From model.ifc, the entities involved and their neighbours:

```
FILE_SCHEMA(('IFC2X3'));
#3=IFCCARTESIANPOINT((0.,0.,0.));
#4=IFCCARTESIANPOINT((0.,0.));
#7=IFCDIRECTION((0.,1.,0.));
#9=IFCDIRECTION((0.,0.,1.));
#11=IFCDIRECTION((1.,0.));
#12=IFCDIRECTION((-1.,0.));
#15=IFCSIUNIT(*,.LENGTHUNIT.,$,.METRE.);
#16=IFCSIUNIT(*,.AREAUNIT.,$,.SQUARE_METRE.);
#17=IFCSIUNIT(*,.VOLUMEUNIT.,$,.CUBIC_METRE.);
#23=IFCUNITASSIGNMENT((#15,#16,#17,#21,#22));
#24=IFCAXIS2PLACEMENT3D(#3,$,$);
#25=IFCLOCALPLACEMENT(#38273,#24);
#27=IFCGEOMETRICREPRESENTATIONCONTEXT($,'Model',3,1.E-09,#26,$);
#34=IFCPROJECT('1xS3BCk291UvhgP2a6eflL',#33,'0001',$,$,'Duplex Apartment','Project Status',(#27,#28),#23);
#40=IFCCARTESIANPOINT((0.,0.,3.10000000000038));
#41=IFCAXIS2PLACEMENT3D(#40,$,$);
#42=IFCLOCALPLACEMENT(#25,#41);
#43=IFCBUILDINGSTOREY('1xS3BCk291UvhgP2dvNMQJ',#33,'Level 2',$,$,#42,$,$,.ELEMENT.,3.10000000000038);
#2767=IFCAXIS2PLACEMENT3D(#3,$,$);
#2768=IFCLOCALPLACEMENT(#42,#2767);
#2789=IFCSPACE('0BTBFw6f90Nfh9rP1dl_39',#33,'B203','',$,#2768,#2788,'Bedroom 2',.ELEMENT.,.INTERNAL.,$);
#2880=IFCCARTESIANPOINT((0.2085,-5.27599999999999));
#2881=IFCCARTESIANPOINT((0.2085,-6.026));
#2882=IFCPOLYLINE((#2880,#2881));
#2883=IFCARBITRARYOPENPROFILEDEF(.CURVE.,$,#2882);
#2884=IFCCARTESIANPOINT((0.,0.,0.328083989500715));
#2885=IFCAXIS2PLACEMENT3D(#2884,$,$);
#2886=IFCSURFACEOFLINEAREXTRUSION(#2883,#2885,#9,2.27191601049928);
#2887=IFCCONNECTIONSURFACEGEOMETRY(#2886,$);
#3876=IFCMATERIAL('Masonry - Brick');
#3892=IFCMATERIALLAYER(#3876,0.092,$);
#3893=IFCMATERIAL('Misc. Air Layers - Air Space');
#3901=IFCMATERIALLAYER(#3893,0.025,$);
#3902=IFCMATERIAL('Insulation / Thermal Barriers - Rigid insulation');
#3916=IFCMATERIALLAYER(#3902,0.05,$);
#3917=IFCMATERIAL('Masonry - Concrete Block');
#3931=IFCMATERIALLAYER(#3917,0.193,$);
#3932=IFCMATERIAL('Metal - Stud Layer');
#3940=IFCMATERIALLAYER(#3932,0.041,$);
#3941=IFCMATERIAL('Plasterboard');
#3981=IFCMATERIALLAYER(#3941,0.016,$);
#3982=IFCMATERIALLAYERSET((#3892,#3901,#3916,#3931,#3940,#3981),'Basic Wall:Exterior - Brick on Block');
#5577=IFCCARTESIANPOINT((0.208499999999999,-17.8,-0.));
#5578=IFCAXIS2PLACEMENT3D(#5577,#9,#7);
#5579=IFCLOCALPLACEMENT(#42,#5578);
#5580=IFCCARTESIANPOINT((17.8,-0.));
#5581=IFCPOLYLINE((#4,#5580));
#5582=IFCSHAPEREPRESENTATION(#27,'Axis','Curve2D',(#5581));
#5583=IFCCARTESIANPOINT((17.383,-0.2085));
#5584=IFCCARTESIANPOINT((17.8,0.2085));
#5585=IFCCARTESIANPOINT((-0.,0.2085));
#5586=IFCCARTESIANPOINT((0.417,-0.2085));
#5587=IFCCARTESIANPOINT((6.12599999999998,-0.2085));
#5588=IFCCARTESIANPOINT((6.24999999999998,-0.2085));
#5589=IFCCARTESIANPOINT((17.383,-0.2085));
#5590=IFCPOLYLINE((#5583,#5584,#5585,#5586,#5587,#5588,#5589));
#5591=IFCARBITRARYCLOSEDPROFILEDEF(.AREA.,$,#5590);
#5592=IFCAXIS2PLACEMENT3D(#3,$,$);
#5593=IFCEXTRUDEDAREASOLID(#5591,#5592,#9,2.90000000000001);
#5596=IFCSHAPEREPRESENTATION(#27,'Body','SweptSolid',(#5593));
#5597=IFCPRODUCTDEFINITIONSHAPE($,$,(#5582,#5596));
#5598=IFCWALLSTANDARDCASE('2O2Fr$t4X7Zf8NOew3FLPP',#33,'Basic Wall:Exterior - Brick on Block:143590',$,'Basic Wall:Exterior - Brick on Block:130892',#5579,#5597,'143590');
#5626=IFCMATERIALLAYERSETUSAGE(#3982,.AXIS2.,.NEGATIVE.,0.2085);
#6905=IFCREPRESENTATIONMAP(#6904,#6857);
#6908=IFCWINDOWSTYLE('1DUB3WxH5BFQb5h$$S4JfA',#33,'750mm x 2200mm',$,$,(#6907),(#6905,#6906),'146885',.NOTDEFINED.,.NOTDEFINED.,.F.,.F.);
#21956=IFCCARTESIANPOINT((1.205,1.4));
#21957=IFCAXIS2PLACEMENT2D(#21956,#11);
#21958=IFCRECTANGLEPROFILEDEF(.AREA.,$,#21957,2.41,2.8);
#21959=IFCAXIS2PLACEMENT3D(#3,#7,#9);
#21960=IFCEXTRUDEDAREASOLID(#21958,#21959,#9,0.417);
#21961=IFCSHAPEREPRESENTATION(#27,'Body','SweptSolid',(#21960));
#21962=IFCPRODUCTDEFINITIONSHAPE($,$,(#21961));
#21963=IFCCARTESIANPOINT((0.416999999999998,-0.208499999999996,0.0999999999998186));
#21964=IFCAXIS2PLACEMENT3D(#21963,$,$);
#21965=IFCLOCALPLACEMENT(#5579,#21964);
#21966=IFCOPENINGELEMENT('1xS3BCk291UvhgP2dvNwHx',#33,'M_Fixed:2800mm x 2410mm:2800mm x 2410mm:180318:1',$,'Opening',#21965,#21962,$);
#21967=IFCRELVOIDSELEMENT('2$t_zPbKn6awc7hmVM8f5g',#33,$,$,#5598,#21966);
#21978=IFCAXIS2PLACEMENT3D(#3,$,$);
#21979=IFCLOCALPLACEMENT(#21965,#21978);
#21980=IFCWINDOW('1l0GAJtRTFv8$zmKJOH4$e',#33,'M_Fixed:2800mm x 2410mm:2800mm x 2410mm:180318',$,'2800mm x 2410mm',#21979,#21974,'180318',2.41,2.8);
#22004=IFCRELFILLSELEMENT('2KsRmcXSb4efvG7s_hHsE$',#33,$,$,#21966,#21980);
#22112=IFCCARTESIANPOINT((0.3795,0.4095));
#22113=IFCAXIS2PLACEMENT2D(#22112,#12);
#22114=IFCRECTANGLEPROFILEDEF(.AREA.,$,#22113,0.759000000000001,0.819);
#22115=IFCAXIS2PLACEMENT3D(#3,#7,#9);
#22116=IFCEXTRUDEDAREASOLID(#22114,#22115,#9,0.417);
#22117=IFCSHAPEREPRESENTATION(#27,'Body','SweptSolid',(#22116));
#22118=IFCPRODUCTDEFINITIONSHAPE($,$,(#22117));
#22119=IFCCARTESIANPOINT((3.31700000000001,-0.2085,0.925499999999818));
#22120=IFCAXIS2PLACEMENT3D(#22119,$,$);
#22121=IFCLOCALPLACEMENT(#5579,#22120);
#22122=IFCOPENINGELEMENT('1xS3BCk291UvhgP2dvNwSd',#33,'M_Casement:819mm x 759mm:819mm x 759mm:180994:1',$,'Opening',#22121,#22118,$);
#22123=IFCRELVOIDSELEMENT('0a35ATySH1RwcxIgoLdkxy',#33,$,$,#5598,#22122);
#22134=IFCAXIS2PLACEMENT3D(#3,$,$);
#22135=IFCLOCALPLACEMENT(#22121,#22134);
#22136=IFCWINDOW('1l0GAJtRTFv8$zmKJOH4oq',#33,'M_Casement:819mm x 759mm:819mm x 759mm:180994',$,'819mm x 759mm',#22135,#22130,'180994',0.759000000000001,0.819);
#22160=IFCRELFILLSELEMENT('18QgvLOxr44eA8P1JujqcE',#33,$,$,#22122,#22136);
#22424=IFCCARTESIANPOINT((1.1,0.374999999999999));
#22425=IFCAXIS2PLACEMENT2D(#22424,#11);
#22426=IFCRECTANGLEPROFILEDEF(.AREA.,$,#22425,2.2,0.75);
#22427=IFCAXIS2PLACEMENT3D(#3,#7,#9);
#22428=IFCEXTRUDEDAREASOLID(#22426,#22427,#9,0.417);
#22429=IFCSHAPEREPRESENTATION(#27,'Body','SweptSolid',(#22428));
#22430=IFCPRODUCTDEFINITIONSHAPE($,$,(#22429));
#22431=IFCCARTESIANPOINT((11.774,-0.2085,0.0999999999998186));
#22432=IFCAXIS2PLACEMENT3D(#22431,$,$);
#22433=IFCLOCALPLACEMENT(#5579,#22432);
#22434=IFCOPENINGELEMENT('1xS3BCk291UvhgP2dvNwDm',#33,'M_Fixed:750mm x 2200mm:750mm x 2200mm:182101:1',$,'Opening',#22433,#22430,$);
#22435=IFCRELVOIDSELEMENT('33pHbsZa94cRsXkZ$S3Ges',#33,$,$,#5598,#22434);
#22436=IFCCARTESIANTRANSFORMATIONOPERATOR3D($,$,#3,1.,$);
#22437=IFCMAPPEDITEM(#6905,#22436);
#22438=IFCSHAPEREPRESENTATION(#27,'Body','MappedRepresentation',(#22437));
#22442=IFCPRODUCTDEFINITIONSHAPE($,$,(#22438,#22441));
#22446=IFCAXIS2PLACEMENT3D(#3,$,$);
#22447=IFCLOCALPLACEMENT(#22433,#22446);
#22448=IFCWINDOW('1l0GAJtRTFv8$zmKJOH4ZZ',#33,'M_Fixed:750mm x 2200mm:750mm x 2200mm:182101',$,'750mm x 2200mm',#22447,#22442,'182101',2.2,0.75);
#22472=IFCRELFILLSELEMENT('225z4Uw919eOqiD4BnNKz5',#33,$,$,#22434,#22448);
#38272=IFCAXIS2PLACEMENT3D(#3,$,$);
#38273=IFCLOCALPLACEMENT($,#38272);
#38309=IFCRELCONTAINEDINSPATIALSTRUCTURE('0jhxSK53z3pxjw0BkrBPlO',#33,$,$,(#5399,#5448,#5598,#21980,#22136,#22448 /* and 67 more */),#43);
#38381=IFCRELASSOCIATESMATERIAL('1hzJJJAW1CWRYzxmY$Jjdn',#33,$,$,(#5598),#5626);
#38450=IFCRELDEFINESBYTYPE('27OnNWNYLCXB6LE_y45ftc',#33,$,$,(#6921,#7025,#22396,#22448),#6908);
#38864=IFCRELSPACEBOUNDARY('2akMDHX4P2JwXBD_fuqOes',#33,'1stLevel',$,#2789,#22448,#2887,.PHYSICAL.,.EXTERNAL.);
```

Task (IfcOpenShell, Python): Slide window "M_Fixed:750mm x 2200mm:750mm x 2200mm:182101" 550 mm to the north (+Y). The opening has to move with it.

```python
import numpy as np
import ifcopenshell
import ifcopenshell.api.geometry
import ifcopenshell.util.placement

model = ifcopenshell.open("model.ifc")

window = model.by_guid("1l0GAJtRTFv8$zmKJOH4ZZ")
opening = window.FillsVoids[0].RelatingOpeningElement
wall = opening.VoidsElements[0].RelatingBuildingElement

wall_matrix = ifcopenshell.util.placement.get_local_placement(wall.ObjectPlacement)
shift = wall_matrix[:3, 0] * 0.55
before = ifcopenshell.util.placement.get_local_placement(window.ObjectPlacement)[:3, 3].copy()

# The window is placed relative to its opening, so it follows when the opening moves.
matrix = ifcopenshell.util.placement.get_local_placement(opening.ObjectPlacement)
matrix[:3, 3] += shift
ifcopenshell.api.geometry.edit_object_placement(
    model, product=opening, matrix=matrix, is_si=False, should_transform_children=True
)

# Space boundary surfaces are stored in each space's coordinates; move them too.
for rel in window.ProvidesBoundaries:
    if not rel.ConnectionGeometry:
        continue
    surface = rel.ConnectionGeometry.SurfaceOnRelatingElement
    space_matrix = ifcopenshell.util.placement.get_local_placement(rel.RelatingSpace.ObjectPlacement)
    point = np.array(surface.Position.Location.Coordinates) + space_matrix[:3, :3].T @ shift
    surface.Position = model.createIfcAxis2Placement3D(
        model.createIfcCartesianPoint(point.tolist()), surface.Position.Axis, surface.Position.RefDirection
    )

after = ifcopenshell.util.placement.get_local_placement(window.ObjectPlacement)[:3, 3]
print("window moved by", (after - before).round(3) + 0.0)

model.write("model-out.ifc")
```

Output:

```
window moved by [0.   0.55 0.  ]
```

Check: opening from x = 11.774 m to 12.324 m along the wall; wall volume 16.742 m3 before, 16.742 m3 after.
